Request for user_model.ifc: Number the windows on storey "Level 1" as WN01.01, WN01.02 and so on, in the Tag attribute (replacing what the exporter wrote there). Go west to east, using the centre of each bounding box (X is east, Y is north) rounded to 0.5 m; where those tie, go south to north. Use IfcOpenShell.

First a look at what the model holds.

```python
import ifcopenshell
import ifcopenshell.util.element
import ifcopenshell.util.placement

model = ifcopenshell.open("user_model.ifc")
print(model.schema)
storey = next(s for s in model.by_type("IfcBuildingStorey") if s.Name == "Level 1")
windows = [e for e in ifcopenshell.util.element.get_decomposition(storey) if e.is_a("IfcWindow")]
for e in sorted(windows, key=lambda e: e.id()):
    origin = ifcopenshell.util.placement.get_local_placement(e.ObjectPlacement)[:3, 3]
    print(e.id(), e.Tag, e.Name, origin.round(2) + 0.0, sep=" | ")
```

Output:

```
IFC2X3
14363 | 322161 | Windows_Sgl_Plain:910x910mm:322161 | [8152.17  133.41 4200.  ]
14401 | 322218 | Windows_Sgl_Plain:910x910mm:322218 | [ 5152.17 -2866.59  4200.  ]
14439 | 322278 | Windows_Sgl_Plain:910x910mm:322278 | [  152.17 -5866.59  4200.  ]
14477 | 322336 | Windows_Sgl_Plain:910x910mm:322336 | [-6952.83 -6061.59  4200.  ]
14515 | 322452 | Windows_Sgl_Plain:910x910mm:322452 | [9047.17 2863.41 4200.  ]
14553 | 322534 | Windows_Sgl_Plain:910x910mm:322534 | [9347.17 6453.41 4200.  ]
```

```python
import ifcopenshell
import ifcopenshell.geom
import ifcopenshell.util.element
import ifcopenshell.util.shape

model = ifcopenshell.open("user_model.ifc")
settings = ifcopenshell.geom.settings()
settings.set("use-world-coords", True)


def centre(element):
    shape = ifcopenshell.geom.create_shape(settings, element)
    return ifcopenshell.util.shape.get_bbox_centroid(shape.geometry)


storey = next(s for s in model.by_type("IfcBuildingStorey") if s.Name == "Level 1")
windows = [e for e in ifcopenshell.util.element.get_decomposition(storey) if e.is_a("IfcWindow")]

# Insertion points can sit at a corner or the storey origin, so sort by the geometry (in metres).
centres = {e: centre(e) for e in windows}
windows.sort(key=lambda e: (round(centres[e][0] / 0.5), centres[e][1]))

for i, e in enumerate(windows, start=1):
    number = f"WN01.{i:02d}"
    e.Tag = number
    print(e.id(), number)

model.write("user_model_edited.ifc")
```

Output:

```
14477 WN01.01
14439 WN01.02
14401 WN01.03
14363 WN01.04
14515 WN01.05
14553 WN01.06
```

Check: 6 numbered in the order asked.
